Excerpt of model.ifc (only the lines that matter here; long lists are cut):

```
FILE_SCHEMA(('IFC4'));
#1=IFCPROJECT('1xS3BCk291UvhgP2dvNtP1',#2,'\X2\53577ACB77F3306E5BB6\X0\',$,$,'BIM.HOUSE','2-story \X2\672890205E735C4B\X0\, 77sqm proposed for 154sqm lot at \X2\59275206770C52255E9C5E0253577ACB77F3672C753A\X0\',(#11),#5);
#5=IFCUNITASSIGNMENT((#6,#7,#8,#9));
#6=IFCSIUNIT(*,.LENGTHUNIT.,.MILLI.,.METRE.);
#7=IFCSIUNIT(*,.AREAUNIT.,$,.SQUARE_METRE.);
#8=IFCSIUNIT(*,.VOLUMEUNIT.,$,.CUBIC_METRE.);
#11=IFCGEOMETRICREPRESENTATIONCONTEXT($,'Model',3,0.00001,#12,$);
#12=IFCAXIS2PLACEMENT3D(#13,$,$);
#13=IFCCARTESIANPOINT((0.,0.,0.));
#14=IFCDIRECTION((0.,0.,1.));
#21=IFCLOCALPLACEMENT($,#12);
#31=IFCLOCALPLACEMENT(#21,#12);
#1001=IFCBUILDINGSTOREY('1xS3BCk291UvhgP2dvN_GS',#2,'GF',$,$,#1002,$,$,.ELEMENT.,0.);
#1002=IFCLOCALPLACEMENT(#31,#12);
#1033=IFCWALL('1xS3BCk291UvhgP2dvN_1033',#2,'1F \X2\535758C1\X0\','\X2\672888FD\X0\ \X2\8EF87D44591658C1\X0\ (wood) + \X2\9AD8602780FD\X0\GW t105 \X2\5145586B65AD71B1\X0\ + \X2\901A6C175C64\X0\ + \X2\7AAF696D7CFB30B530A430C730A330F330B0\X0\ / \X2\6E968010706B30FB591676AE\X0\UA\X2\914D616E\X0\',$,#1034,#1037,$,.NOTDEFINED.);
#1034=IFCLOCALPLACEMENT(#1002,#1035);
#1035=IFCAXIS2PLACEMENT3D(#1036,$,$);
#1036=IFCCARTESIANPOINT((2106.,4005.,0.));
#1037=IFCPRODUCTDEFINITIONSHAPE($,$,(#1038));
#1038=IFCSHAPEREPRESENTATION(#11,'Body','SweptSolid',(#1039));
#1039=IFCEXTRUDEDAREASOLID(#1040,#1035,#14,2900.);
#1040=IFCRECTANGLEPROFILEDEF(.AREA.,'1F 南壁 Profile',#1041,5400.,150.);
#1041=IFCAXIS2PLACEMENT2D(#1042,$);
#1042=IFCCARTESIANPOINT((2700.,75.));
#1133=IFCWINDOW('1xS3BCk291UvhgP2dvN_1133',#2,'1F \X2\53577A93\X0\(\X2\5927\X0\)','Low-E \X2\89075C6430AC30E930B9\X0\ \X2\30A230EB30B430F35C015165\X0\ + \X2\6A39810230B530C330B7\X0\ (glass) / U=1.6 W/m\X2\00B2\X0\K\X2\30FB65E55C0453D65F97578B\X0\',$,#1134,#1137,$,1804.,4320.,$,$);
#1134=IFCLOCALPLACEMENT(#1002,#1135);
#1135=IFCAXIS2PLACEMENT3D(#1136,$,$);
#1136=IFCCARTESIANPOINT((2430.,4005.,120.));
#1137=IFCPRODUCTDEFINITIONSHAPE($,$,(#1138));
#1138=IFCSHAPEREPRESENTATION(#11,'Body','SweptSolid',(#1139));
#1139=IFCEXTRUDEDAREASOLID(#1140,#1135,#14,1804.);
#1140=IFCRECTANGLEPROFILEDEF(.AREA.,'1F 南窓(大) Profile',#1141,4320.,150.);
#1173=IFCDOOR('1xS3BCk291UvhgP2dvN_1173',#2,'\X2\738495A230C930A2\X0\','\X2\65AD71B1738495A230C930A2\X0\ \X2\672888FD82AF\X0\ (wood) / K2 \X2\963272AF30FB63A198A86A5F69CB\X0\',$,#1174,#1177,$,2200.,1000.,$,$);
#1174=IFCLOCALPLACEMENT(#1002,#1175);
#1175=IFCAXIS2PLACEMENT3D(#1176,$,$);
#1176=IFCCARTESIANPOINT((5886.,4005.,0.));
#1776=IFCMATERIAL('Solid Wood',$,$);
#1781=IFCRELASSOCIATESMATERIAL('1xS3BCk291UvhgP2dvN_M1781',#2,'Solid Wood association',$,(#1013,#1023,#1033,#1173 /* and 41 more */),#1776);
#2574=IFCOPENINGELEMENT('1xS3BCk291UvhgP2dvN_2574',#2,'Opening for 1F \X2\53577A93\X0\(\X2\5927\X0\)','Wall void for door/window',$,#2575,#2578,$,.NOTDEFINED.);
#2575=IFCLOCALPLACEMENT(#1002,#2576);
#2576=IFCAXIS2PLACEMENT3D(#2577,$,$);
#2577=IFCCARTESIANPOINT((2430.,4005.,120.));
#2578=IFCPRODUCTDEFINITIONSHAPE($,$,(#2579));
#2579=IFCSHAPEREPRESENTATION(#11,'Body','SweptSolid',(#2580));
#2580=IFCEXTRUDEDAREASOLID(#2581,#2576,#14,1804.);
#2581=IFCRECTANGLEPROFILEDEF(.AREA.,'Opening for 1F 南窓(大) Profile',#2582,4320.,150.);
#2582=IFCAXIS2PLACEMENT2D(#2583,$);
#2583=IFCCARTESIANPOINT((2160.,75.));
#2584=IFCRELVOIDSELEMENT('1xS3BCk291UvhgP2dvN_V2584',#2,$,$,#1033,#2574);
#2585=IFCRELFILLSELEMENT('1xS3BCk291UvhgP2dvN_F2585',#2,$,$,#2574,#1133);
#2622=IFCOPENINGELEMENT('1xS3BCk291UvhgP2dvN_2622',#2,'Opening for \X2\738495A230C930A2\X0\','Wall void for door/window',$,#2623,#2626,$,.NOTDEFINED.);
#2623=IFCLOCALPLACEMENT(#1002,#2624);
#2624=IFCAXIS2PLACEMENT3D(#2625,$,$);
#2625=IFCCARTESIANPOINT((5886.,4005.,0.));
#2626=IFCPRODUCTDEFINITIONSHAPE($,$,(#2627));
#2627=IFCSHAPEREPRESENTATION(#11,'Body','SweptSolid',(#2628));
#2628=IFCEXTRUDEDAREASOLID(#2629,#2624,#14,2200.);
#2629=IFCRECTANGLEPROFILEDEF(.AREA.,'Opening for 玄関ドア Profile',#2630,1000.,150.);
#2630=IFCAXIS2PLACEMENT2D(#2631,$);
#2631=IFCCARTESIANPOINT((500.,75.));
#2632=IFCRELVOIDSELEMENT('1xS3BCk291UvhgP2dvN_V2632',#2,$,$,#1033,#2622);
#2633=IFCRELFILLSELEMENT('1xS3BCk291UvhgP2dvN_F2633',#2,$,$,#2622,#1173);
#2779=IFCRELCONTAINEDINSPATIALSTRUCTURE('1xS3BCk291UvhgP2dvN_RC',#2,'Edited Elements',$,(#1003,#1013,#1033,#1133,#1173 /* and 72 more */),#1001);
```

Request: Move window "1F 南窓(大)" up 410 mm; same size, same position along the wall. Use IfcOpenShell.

```python
import numpy as np
import ifcopenshell
import ifcopenshell.api.geometry
import ifcopenshell.util.placement
import ifcopenshell.util.unit

model = ifcopenshell.open("model.ifc")
unit_scale = ifcopenshell.util.unit.calculate_unit_scale(model)

window = model.by_guid("1xS3BCk291UvhgP2dvN_1133")
opening = window.FillsVoids[0].RelatingOpeningElement
dz = 0.41 / unit_scale

shift = np.array([0.0, 0.0, dz])
# The window is not placed relative to its opening, so move both.
for product in (opening, window):
    matrix = ifcopenshell.util.placement.get_local_placement(product.ObjectPlacement)
    matrix[:3, 3] += shift
    ifcopenshell.api.geometry.edit_object_placement(model, product=product, matrix=matrix, is_si=False)

print(f"moved by {dz * unit_scale:+.3f} m")

model.write("model_updated.ifc")
```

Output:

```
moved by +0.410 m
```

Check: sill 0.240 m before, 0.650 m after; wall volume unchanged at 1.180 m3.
